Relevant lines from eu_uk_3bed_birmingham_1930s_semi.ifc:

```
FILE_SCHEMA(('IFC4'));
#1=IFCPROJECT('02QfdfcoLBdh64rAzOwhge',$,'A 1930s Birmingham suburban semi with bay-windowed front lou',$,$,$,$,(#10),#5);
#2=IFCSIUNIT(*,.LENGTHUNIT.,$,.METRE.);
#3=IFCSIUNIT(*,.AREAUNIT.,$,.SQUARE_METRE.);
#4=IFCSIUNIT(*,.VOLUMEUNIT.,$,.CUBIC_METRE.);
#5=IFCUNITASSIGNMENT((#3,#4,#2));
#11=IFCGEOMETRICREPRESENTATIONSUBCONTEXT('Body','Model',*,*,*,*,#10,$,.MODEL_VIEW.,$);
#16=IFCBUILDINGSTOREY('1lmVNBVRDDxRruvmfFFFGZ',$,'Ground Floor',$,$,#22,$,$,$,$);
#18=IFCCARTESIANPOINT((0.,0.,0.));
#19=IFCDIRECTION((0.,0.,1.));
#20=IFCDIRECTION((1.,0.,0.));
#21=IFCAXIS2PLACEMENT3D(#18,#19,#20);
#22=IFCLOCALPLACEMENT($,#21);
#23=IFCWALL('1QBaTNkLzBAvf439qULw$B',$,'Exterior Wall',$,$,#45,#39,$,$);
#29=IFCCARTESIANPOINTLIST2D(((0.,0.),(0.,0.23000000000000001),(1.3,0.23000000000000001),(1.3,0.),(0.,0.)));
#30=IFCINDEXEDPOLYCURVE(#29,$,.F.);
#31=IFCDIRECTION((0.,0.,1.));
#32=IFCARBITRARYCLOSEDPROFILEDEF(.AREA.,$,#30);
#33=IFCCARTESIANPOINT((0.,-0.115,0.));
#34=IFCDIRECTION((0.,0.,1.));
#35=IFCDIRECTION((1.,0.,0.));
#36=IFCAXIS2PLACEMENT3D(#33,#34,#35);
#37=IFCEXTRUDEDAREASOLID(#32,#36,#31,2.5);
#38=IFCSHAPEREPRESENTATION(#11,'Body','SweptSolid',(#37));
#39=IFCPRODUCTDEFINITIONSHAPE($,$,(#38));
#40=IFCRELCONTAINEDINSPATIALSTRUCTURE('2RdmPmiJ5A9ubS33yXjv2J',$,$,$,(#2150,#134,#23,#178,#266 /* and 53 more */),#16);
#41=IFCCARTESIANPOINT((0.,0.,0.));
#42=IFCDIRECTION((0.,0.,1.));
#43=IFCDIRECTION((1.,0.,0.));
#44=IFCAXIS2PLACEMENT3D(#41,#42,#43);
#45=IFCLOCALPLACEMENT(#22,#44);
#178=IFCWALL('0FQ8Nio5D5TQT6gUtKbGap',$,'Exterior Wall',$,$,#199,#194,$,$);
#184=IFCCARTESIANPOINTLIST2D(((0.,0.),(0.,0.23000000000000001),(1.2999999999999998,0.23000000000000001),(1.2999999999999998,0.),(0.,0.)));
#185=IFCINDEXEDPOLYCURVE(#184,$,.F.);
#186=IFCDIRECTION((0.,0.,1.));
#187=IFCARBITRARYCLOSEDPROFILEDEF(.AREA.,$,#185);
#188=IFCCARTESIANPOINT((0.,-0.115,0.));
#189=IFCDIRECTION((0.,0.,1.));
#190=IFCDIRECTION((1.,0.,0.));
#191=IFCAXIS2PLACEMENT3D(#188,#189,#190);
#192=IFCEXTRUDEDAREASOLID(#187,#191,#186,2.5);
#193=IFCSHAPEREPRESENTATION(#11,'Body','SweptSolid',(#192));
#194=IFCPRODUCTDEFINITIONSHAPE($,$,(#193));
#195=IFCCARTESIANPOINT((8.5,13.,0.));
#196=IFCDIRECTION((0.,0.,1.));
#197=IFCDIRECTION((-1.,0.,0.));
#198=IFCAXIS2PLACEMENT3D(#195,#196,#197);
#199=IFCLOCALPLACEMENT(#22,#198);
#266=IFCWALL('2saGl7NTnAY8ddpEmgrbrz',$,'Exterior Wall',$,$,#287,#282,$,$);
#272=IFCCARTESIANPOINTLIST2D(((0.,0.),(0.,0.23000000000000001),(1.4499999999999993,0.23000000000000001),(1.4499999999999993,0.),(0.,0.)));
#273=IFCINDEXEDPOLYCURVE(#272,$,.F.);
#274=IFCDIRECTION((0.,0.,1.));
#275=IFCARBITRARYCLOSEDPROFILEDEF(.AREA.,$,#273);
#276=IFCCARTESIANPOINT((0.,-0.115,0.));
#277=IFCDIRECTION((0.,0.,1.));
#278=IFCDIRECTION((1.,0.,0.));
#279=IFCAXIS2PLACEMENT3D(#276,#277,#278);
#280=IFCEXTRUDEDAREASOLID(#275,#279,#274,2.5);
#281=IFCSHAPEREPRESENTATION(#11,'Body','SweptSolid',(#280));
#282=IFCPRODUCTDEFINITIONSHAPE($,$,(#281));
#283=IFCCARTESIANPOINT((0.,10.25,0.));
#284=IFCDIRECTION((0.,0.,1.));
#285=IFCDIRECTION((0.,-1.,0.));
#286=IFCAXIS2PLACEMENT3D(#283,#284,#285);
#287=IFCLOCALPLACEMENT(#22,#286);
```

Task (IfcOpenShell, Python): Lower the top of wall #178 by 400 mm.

```python
import ifcopenshell
import ifcopenshell.geom
import ifcopenshell.util.representation
import ifcopenshell.util.shape
import ifcopenshell.util.unit

model = ifcopenshell.open("eu_uk_3bed_birmingham_1930s_semi.ifc")
unit_scale = ifcopenshell.util.unit.calculate_unit_scale(model)
settings = ifcopenshell.geom.settings()


def volume(element):
    """Net volume in cubic metres, openings subtracted."""
    shape = ifcopenshell.geom.create_shape(settings, element)
    return ifcopenshell.util.shape.get_volume(shape.geometry)


wall = model.by_guid("0FQ8Nio5D5TQT6gUtKbGap")
before = volume(wall)

body = ifcopenshell.util.representation.get_representation(wall, "Model", "Body")
solid = body.Items[0]
old_height = solid.Depth
solid.Depth -= 0.4 / unit_scale
after = volume(wall)

print(f"height {old_height:g} -> {solid.Depth:g}, volume {before:.3f} -> {after:.3f} m3")

model.write("eu_uk_3bed_birmingham_1930s_semi-out.ifc")
```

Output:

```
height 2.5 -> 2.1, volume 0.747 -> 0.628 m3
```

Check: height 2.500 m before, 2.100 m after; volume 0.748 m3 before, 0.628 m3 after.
